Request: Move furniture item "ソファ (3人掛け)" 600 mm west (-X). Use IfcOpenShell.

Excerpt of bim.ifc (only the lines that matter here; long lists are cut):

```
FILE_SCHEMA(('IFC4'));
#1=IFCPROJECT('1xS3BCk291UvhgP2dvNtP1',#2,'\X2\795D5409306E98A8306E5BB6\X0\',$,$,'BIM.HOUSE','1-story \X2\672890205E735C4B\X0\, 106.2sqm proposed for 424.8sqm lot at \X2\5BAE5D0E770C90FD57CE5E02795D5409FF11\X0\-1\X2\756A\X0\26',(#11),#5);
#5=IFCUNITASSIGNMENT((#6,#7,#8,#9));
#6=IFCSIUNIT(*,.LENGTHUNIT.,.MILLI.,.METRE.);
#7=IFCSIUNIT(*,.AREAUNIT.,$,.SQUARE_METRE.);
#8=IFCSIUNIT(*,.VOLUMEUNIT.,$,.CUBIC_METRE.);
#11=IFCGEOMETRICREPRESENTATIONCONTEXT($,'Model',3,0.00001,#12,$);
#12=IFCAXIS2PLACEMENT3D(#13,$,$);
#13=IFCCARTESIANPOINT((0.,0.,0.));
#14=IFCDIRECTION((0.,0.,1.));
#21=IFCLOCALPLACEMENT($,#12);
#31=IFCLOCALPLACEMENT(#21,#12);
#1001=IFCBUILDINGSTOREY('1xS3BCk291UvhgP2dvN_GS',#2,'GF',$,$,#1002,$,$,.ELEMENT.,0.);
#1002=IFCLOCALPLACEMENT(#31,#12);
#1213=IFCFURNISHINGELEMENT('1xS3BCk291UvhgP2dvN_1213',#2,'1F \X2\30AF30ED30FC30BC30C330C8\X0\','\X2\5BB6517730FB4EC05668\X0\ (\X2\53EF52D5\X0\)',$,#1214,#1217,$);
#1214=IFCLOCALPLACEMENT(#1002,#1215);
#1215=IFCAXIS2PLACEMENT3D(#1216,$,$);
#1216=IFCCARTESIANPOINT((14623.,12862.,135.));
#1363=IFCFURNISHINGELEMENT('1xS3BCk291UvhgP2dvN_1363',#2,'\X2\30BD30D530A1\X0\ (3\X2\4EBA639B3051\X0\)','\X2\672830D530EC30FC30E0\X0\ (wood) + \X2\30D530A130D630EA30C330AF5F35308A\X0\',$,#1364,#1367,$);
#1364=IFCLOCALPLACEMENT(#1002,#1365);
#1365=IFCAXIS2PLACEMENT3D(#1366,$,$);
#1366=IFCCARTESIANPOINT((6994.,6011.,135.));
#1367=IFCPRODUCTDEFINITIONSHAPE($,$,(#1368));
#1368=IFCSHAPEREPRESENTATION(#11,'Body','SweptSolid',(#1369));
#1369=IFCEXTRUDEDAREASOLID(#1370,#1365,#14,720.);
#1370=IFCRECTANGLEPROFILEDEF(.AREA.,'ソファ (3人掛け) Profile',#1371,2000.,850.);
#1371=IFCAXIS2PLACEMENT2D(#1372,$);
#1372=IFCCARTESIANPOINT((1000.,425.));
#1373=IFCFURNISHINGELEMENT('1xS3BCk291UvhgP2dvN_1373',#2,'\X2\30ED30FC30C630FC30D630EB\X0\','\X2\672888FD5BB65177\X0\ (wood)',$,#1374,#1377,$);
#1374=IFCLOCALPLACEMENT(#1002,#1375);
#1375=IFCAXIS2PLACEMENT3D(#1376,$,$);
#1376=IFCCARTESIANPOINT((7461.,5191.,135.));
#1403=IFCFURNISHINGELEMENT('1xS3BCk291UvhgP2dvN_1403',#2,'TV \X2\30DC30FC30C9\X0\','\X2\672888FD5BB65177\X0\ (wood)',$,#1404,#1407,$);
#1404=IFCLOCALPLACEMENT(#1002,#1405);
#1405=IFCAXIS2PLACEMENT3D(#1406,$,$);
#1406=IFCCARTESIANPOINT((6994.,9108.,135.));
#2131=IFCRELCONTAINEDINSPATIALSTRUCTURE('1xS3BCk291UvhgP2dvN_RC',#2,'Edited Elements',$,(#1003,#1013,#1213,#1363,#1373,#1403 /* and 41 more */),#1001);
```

```python
import ifcopenshell
import ifcopenshell.api.geometry
import ifcopenshell.util.placement

model = ifcopenshell.open("bim.ifc")

item = model.by_id(1363)
matrix = ifcopenshell.util.placement.get_local_placement(item.ObjectPlacement)
matrix[0, 3] -= 600.0
ifcopenshell.api.geometry.edit_object_placement(model, product=item, matrix=matrix, is_si=False)

print(ifcopenshell.util.placement.get_local_placement(item.ObjectPlacement).round(3) + 0.0)

model.write("bim_rev.ifc")
```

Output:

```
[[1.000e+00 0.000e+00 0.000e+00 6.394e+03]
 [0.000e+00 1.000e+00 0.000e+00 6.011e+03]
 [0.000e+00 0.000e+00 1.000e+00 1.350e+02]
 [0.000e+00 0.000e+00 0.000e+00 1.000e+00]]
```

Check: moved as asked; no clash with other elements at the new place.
